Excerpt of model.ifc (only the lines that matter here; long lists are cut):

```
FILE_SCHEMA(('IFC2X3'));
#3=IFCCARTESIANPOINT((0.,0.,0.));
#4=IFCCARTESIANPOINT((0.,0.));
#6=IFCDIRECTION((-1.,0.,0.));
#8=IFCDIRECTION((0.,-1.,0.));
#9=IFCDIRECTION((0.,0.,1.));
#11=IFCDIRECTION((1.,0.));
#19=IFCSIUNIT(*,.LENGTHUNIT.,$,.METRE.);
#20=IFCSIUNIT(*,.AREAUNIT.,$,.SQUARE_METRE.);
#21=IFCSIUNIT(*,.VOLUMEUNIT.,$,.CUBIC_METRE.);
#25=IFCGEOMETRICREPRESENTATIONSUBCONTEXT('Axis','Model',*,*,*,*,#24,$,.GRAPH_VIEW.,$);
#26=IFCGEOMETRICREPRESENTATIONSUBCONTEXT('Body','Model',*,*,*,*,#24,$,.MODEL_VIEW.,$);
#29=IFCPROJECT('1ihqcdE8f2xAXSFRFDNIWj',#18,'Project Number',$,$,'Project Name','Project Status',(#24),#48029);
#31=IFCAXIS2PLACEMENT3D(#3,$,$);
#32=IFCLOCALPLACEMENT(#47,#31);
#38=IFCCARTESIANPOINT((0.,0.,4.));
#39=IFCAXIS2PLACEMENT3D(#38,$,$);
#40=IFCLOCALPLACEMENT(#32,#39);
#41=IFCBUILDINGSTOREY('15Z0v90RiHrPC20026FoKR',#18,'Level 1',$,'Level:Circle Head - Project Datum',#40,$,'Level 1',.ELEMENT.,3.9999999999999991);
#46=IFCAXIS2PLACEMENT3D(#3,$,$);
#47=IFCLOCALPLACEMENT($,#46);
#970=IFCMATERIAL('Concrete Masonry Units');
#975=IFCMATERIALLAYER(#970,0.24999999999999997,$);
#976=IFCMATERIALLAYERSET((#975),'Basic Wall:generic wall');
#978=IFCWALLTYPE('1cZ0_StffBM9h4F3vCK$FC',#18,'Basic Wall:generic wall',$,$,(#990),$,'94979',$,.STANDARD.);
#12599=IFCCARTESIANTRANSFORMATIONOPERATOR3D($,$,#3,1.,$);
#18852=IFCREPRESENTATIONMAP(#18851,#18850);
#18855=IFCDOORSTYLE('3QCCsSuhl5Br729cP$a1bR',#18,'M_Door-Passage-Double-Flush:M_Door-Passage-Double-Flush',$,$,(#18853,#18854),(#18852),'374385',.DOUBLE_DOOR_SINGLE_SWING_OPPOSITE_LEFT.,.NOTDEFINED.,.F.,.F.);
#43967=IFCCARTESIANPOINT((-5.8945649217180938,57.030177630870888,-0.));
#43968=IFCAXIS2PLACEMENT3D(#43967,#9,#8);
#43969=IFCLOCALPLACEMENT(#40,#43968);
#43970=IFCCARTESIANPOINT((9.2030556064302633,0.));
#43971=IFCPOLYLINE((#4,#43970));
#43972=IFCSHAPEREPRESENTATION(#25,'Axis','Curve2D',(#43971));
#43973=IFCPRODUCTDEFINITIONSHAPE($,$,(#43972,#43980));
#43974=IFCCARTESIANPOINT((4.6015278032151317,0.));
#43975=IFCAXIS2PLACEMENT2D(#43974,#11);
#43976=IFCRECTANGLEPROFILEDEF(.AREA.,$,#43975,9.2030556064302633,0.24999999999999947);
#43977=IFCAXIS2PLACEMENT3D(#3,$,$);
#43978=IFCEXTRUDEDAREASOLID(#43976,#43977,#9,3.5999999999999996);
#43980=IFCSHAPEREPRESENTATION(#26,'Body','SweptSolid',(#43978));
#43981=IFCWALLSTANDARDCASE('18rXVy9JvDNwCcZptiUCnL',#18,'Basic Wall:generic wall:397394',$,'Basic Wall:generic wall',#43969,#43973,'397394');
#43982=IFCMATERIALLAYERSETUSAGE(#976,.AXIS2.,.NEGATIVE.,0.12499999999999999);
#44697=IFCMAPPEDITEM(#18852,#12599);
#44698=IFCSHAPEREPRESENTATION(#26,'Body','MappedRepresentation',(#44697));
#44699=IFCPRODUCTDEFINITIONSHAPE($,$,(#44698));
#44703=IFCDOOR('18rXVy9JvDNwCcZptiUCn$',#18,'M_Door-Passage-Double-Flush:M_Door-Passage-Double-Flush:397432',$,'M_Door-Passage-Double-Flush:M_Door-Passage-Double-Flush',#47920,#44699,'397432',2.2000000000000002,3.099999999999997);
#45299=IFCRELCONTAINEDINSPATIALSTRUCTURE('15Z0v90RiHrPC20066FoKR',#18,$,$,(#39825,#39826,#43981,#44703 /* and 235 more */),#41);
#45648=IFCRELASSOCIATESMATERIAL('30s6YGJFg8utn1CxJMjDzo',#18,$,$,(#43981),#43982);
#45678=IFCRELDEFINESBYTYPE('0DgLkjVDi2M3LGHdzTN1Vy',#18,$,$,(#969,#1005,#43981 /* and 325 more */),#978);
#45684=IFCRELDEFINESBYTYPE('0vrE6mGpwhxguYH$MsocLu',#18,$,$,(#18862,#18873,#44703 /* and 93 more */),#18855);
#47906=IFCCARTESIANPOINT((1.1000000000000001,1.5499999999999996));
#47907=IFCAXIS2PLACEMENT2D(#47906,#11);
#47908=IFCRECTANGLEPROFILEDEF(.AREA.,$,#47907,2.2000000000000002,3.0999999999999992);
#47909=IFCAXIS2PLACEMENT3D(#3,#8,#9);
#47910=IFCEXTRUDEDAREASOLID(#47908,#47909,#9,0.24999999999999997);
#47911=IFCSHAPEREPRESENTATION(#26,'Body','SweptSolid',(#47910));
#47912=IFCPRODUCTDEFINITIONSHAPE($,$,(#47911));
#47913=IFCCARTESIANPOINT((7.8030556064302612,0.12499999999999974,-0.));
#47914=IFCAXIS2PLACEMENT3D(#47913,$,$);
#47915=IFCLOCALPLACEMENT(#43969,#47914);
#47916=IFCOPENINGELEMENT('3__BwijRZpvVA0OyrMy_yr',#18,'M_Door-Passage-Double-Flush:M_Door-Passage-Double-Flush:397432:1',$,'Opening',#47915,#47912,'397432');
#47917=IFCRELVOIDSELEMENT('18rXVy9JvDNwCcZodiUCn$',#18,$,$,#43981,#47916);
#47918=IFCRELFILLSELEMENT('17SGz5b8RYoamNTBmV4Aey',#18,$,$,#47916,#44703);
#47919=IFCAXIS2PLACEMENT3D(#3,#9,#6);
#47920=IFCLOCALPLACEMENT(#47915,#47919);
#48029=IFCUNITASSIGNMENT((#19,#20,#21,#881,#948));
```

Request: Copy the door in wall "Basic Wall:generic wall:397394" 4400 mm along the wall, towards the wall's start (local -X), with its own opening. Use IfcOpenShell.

```python
import ifcopenshell
import ifcopenshell.api.feature
import ifcopenshell.api.geometry
import ifcopenshell.api.root
import ifcopenshell.geom
import ifcopenshell.util.element
import ifcopenshell.util.placement
import ifcopenshell.util.shape

model = ifcopenshell.open("model.ifc")
settings = ifcopenshell.geom.settings()


def volume(element):
    """Net volume in cubic metres, openings subtracted."""
    shape = ifcopenshell.geom.create_shape(settings, element)
    return ifcopenshell.util.shape.get_volume(shape.geometry)


def reuse_history(source, copy):
    """copy_class also copies each property set's owner history, people and application; keep the originals."""
    for rel in copy.IsDefinedBy:
        if rel.is_a("IfcRelDefinesByProperties") and (history := rel.RelatingPropertyDefinition.OwnerHistory):
            rel.RelatingPropertyDefinition.OwnerHistory = source.OwnerHistory
            ifcopenshell.util.element.remove_deep2(model, history)


door = model.by_id(44703)
opening = door.FillsVoids[0].RelatingOpeningElement
wall = opening.VoidsElements[0].RelatingBuildingElement
before = volume(wall)
shift = ifcopenshell.util.placement.get_local_placement(wall.ObjectPlacement)[:3, 0] * -4.4

# copy_class copies the void relationship, type, container and properties, but no geometry.
new_opening = ifcopenshell.api.root.copy_class(model, product=opening)
new_opening.Representation = ifcopenshell.util.element.copy_deep(
    model, opening.Representation, exclude=["IfcGeometricRepresentationContext", "IfcRepresentationMap"]
)
new_opening.Name = "M_Door-Passage-Double-Flush:M_Door-Passage-Double-Flush"
new_opening.Tag = None
new_door = ifcopenshell.api.root.copy_class(model, product=door)
new_door.Representation = ifcopenshell.util.element.copy_deep(
    model, door.Representation, exclude=["IfcGeometricRepresentationContext", "IfcRepresentationMap"]
)
new_door.Name = "M_Door-Passage-Double-Flush:M_Door-Passage-Double-Flush"
new_door.Tag = None
reuse_history(door, new_door)
fills = ifcopenshell.api.feature.add_filling(model, opening=new_opening, element=new_door)
fills.OwnerHistory = new_door.OwnerHistory  # required in IFC2X3

for old, new in ((opening, new_opening), (door, new_door)):
    matrix = ifcopenshell.util.placement.get_local_placement(old.ObjectPlacement)
    matrix[:3, 3] += shift
    ifcopenshell.api.geometry.edit_object_placement(model, product=new, matrix=matrix, is_si=False)

after = volume(wall)

print(f"wall volume {before:.3f} -> {after:.3f} m3")

model.write("model_edited.ifc")
```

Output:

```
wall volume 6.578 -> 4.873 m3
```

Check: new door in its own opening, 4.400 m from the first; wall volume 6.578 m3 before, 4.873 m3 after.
